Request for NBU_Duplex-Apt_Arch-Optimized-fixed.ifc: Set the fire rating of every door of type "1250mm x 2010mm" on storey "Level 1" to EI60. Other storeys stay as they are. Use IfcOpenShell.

First a look at what the model holds.

```python
import ifcopenshell
import ifcopenshell.util.element

model = ifcopenshell.open("NBU_Duplex-Apt_Arch-Optimized-fixed.ifc")
print(model.schema)
storey = next(s for s in model.by_type("IfcBuildingStorey") if s.Name == "Level 1")
doors = [e for e in ifcopenshell.util.element.get_decomposition(storey) if e.is_a("IfcDoor")]
seen = {}
for e in doors:
    element_type = ifcopenshell.util.element.get_type(e)
    key = (element_type.Name if element_type != e and element_type else None, ifcopenshell.util.element.get_pset(e, "Pset_DoorCommon", "FireRating"))
    seen[key] = seen.get(key, 0) + 1
for (name, value), count in sorted(seen.items(), key=str):
    print(count, "x", name, "|", value)
```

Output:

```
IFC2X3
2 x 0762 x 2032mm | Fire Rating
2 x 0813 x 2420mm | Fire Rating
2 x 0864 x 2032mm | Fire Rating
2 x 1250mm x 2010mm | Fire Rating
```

```python
import ifcopenshell
import ifcopenshell.api.pset
import ifcopenshell.util.element

model = ifcopenshell.open("NBU_Duplex-Apt_Arch-Optimized-fixed.ifc")

storey = next(s for s in model.by_type("IfcBuildingStorey") if s.Name == "Level 1")
doors = [e for e in ifcopenshell.util.element.get_decomposition(storey) if e.is_a("IfcDoor")]

count = 0
for e in doors:
    element_type = ifcopenshell.util.element.get_type(e)
    if element_type in (None, e) or element_type.Name != "1250mm x 2010mm":
        continue
    # add_pset returns the element's existing set when there is one.
    pset = ifcopenshell.api.pset.add_pset(model, product=e, name="Pset_DoorCommon")
    ifcopenshell.api.pset.edit_pset(model, pset=pset, properties={"FireRating": "EI60"})
    count += 1

print(count, "doors updated")

model.write("NBU_Duplex-Apt_Arch-Optimized-fixed_v2.ifc")
```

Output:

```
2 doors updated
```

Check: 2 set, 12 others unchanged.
